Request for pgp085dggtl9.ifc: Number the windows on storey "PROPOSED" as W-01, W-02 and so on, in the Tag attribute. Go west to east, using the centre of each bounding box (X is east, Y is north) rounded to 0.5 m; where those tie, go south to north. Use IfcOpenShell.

First a look at what the model holds.

```python
import ifcopenshell
import ifcopenshell.util.element
import ifcopenshell.util.placement

model = ifcopenshell.open("pgp085dggtl9.ifc")
print(model.schema)
storey = next(s for s in model.by_type("IfcBuildingStorey") if s.Name == "PROPOSED")
windows = [e for e in ifcopenshell.util.element.get_decomposition(storey) if e.is_a("IfcWindow")]
for e in sorted(windows, key=lambda e: e.id()):
    origin = ifcopenshell.util.placement.get_local_placement(e.ObjectPlacement)[:3, 3]
    print(e.id(), e.Tag, e.Name, origin.round(2) + 0.0, sep=" | ")
```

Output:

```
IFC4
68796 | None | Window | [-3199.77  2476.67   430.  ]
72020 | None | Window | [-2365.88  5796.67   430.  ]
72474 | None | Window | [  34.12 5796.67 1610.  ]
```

```python
import ifcopenshell
import ifcopenshell.geom
import ifcopenshell.util.element
import ifcopenshell.util.shape

model = ifcopenshell.open("pgp085dggtl9.ifc")
settings = ifcopenshell.geom.settings()
settings.set("use-world-coords", True)


def centre(element):
    shape = ifcopenshell.geom.create_shape(settings, element)
    return ifcopenshell.util.shape.get_bbox_centroid(shape.geometry)


storey = next(s for s in model.by_type("IfcBuildingStorey") if s.Name == "PROPOSED")
windows = [e for e in ifcopenshell.util.element.get_decomposition(storey) if e.is_a("IfcWindow")]

# Insertion points can sit at a corner or the storey origin, so sort by the geometry (in metres).
centres = {e: centre(e) for e in windows}
windows.sort(key=lambda e: (round(centres[e][0] / 0.5), centres[e][1]))

for i, e in enumerate(windows, start=1):
    number = f"W-{i:02d}"
    e.Tag = number
    print(e.id(), number)

model.write("pgp085dggtl9_updated.ifc")
```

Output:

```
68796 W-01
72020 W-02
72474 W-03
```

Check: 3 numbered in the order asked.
